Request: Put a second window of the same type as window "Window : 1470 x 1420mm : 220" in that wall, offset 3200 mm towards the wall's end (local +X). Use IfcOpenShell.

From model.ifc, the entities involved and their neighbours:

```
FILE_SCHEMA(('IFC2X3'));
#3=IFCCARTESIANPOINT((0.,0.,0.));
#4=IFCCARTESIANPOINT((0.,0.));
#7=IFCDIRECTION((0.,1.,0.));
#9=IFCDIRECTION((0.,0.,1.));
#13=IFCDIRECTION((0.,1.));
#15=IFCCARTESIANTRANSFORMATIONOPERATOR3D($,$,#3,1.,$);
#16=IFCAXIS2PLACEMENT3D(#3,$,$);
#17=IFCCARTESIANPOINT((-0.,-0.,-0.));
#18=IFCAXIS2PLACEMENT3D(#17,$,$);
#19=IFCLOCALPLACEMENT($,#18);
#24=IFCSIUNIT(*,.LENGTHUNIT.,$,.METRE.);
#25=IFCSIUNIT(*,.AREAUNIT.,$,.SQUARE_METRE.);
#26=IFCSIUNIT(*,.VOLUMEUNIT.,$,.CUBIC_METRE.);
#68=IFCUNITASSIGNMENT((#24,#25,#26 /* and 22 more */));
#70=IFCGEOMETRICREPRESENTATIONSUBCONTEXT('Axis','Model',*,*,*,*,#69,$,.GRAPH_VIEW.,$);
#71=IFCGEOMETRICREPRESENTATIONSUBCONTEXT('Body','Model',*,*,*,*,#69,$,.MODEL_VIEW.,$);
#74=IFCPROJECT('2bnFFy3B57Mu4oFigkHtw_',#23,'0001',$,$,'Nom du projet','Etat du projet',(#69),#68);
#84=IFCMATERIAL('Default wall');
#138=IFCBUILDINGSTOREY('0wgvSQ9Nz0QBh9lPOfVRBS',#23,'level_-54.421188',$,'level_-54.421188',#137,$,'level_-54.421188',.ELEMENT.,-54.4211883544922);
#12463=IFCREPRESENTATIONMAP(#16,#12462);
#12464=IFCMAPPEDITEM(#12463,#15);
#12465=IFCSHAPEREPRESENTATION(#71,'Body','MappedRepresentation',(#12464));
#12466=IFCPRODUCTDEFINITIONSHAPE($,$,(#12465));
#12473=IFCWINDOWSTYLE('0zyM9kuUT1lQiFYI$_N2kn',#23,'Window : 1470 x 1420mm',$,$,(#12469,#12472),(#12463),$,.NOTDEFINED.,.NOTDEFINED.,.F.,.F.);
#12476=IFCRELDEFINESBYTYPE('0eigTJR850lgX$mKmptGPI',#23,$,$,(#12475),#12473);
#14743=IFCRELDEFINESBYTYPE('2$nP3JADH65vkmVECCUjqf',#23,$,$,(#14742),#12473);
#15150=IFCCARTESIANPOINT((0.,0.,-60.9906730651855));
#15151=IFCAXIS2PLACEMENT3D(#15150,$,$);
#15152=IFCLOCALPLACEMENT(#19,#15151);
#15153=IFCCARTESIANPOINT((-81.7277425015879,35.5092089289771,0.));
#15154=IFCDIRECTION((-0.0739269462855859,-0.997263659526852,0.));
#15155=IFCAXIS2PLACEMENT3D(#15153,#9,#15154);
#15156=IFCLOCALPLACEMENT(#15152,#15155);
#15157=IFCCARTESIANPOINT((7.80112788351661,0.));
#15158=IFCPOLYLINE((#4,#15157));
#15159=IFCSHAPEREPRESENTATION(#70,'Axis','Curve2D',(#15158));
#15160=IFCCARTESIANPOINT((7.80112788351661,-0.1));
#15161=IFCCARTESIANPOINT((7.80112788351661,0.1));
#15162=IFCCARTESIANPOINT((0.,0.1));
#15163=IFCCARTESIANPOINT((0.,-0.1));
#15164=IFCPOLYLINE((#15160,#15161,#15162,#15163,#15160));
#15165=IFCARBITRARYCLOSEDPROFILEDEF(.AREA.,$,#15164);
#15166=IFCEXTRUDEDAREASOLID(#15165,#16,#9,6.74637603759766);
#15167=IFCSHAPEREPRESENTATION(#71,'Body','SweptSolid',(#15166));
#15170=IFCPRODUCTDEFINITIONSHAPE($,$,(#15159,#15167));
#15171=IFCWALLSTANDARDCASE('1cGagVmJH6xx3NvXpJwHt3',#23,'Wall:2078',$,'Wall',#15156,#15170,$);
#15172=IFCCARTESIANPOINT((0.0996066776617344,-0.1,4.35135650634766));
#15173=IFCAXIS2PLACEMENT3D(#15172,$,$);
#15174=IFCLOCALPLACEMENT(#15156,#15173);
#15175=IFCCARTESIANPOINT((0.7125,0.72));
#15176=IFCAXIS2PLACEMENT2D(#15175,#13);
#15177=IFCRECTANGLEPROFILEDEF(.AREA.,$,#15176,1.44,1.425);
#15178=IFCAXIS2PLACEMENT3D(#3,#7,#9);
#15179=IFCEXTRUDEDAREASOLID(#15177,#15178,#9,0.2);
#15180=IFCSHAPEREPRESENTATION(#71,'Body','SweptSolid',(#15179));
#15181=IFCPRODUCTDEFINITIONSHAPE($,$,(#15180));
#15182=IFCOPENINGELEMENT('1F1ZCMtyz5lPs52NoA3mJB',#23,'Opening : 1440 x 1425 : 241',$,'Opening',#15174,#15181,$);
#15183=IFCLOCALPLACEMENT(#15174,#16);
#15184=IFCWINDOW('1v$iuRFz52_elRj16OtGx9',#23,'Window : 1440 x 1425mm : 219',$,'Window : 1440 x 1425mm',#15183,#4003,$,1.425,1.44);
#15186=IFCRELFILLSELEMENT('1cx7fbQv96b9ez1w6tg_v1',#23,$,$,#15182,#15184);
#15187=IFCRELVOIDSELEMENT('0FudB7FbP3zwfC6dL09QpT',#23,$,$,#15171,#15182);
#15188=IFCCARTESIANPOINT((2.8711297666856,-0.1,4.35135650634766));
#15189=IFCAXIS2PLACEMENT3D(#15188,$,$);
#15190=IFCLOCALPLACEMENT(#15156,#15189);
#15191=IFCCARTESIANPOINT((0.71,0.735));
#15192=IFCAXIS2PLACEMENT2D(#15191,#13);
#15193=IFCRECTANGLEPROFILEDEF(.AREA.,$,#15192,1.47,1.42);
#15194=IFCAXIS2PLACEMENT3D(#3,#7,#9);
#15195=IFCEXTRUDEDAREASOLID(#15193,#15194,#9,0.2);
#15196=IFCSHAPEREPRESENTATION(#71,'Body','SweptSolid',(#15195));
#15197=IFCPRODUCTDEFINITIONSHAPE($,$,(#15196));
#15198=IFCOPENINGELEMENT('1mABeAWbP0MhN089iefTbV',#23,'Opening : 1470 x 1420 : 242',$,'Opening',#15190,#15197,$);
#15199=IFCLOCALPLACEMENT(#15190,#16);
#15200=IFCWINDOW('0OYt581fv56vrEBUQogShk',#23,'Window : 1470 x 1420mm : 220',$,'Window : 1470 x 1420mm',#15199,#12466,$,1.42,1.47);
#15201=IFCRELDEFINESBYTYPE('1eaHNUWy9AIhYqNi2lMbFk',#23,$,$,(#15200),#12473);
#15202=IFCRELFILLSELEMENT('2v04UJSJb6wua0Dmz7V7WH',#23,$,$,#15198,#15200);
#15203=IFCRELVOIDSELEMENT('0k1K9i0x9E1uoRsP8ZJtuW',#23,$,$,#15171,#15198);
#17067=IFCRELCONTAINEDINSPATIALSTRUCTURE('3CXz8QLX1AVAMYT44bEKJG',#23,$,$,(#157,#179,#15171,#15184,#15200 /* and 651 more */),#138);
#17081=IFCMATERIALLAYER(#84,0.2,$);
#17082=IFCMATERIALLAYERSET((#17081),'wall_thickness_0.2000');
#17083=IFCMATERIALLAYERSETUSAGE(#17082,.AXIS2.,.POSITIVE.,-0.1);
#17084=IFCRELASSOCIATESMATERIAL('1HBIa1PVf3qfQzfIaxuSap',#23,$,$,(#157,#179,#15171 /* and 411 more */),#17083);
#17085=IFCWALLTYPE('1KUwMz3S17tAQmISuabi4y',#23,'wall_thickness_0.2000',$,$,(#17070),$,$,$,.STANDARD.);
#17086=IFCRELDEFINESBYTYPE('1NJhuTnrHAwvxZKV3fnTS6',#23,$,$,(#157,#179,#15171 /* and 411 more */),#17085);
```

```python
import ifcopenshell
import ifcopenshell.api.feature
import ifcopenshell.api.geometry
import ifcopenshell.api.root
import ifcopenshell.geom
import ifcopenshell.util.element
import ifcopenshell.util.placement
import ifcopenshell.util.shape
import ifcopenshell.util.unit

model = ifcopenshell.open("model.ifc")
unit_scale = ifcopenshell.util.unit.calculate_unit_scale(model)
settings = ifcopenshell.geom.settings()


def volume(element):
    """Net volume in cubic metres, openings subtracted."""
    shape = ifcopenshell.geom.create_shape(settings, element)
    return ifcopenshell.util.shape.get_volume(shape.geometry)


window = model.by_id(15200)
opening = window.FillsVoids[0].RelatingOpeningElement
wall = opening.VoidsElements[0].RelatingBuildingElement
before = volume(wall)
shift = ifcopenshell.util.placement.get_local_placement(wall.ObjectPlacement)[:3, 0] * 3.2 / unit_scale

# copy_class copies the void relationship, type, container and properties, but no geometry.
new_opening = ifcopenshell.api.root.copy_class(model, product=opening)
new_opening.Representation = ifcopenshell.util.element.copy_deep(
    model, opening.Representation, exclude=["IfcGeometricRepresentationContext", "IfcRepresentationMap"]
)
new_opening.Name = "Opening : 1470 x 1420"
new_window = ifcopenshell.api.root.copy_class(model, product=window)
new_window.Representation = ifcopenshell.util.element.copy_deep(
    model, window.Representation, exclude=["IfcGeometricRepresentationContext", "IfcRepresentationMap"]
)
new_window.Name = "Window : 1470 x 1420mm"
fills = ifcopenshell.api.feature.add_filling(model, opening=new_opening, element=new_window)
fills.OwnerHistory = new_window.OwnerHistory  # required in IFC2X3

for old, new in ((opening, new_opening), (window, new_window)):
    matrix = ifcopenshell.util.placement.get_local_placement(old.ObjectPlacement)
    matrix[:3, 3] += shift
    ifcopenshell.api.geometry.edit_object_placement(model, product=new, matrix=matrix, is_si=False)

after = volume(wall)

print(f"wall volume {before:.3f} -> {after:.3f} m3")

model.write("model_edited.ifc")
```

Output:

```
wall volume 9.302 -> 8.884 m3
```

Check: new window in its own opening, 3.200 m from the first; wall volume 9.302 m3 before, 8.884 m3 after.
